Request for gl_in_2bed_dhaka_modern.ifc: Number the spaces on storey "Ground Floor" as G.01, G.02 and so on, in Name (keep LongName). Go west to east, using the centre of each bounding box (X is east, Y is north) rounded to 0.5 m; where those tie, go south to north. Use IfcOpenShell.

First a look at what the model holds.

```python
import ifcopenshell
import ifcopenshell.util.element
import ifcopenshell.util.placement

model = ifcopenshell.open("gl_in_2bed_dhaka_modern.ifc")
print(model.schema)
storey = next(s for s in model.by_type("IfcBuildingStorey") if s.Name == "Ground Floor")
spaces = [e for e in ifcopenshell.util.element.get_decomposition(storey) if e.is_a("IfcSpace")]
for e in sorted(spaces, key=lambda e: e.id()):
    origin = ifcopenshell.util.placement.get_local_placement(e.ObjectPlacement)[:3, 3]
    print(e.id(), e.Name, e.LongName, origin.round(2) + 0.0, sep=" | ")
```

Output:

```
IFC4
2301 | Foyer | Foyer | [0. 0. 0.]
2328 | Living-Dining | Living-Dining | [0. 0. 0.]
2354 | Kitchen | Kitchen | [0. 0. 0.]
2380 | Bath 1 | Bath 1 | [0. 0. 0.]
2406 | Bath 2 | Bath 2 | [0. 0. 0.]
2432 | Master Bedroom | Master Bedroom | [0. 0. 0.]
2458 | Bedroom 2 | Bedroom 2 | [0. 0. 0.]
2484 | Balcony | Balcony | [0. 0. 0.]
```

```python
import ifcopenshell
import ifcopenshell.geom
import ifcopenshell.util.element
import ifcopenshell.util.shape

model = ifcopenshell.open("gl_in_2bed_dhaka_modern.ifc")
settings = ifcopenshell.geom.settings()
settings.set("use-world-coords", True)


def centre(element):
    shape = ifcopenshell.geom.create_shape(settings, element)
    return ifcopenshell.util.shape.get_bbox_centroid(shape.geometry)


storey = next(s for s in model.by_type("IfcBuildingStorey") if s.Name == "Ground Floor")
spaces = [e for e in ifcopenshell.util.element.get_decomposition(storey) if e.is_a("IfcSpace")]

# Insertion points can sit at a corner or the storey origin, so sort by the geometry (in metres).
centres = {e: centre(e) for e in spaces}
spaces.sort(key=lambda e: (round(centres[e][0] / 0.5), centres[e][1]))

for i, e in enumerate(spaces, start=1):
    number = f"G.{i:02d}"
    e.Name = number
    print(e.id(), number)

model.write("gl_in_2bed_dhaka_modern_updated.ifc")
```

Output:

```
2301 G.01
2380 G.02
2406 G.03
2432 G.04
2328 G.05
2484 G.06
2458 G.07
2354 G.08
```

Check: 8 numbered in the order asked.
